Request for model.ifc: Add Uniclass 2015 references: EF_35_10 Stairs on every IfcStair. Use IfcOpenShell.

First a look at what the model holds.

```python
import ifcopenshell

model = ifcopenshell.open("model.ifc")
print(model.schema)
print("classifications:", [c.Name for c in model.by_type("IfcClassification")])
for ifc_class in ("IfcDoor", "IfcRoof", "IfcStair", "IfcWall", "IfcWindow"):
    print(ifc_class, len(model.by_type(ifc_class)))
```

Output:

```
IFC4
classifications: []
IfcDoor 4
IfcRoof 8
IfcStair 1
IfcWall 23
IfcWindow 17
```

```python
import ifcopenshell
import ifcopenshell.api.classification

model = ifcopenshell.open("model.ifc")

system = ifcopenshell.api.classification.add_classification(model, classification="Uniclass 2015")

codes = {
    "IfcStair": ("EF_35_10", "Stairs"),
}
for ifc_class, (code, name) in codes.items():
    products = model.by_type(ifc_class)
    ifcopenshell.api.classification.add_reference(
        model, products=products, classification=system, identification=code, name=name
    )
    print(code, len(products))

model.write("model_rev.ifc")
```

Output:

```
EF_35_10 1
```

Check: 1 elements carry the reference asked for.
